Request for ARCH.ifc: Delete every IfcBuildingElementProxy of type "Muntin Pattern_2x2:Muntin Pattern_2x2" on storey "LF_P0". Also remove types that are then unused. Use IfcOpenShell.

First a look at what the model holds.

```python
import ifcopenshell
import ifcopenshell.util.element

model = ifcopenshell.open("ARCH.ifc")
print(model.schema)
storey = next(s for s in model.by_type("IfcBuildingStorey") if s.Name == "LF_P0")
proxies = [e for e in ifcopenshell.util.element.get_decomposition(storey) if e.is_a("IfcBuildingElementProxy")]
seen = {}
for e in proxies:
    element_type = ifcopenshell.util.element.get_type(e)
    name = element_type.Name if element_type not in (None, e) else None
    seen[name] = seen.get(name, 0) + 1
for name, count in sorted(seen.items(), key=str):
    print(count, "x", name)
```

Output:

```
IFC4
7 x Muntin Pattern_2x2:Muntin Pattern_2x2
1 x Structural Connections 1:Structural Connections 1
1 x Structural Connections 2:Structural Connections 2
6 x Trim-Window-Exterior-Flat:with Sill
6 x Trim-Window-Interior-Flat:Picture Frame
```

```python
import ifcopenshell
import ifcopenshell.api.root
import ifcopenshell.util.element

model = ifcopenshell.open("ARCH.ifc")

storey = next(s for s in model.by_type("IfcBuildingStorey") if s.Name == "LF_P0")
proxies = [e for e in ifcopenshell.util.element.get_decomposition(storey) if e.is_a("IfcBuildingElementProxy")]
targets = [e for e in proxies if (t := ifcopenshell.util.element.get_type(e)) not in (None, e) and t.Name == "Muntin Pattern_2x2:Muntin Pattern_2x2"]
types = {ifcopenshell.util.element.get_type(e) for e in targets} - {None, *targets}

for e in targets:
    ifcopenshell.api.root.remove_product(model, product=e)
print(len(targets), "removed")

unused = [t for t in types if not ifcopenshell.util.element.get_types(t)]
for t in unused:
    ifcopenshell.api.root.remove_product(model, product=t)
print(len(unused), "unused types removed")

model.write("ARCH_v2.ifc")
```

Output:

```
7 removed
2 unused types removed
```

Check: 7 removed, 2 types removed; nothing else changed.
